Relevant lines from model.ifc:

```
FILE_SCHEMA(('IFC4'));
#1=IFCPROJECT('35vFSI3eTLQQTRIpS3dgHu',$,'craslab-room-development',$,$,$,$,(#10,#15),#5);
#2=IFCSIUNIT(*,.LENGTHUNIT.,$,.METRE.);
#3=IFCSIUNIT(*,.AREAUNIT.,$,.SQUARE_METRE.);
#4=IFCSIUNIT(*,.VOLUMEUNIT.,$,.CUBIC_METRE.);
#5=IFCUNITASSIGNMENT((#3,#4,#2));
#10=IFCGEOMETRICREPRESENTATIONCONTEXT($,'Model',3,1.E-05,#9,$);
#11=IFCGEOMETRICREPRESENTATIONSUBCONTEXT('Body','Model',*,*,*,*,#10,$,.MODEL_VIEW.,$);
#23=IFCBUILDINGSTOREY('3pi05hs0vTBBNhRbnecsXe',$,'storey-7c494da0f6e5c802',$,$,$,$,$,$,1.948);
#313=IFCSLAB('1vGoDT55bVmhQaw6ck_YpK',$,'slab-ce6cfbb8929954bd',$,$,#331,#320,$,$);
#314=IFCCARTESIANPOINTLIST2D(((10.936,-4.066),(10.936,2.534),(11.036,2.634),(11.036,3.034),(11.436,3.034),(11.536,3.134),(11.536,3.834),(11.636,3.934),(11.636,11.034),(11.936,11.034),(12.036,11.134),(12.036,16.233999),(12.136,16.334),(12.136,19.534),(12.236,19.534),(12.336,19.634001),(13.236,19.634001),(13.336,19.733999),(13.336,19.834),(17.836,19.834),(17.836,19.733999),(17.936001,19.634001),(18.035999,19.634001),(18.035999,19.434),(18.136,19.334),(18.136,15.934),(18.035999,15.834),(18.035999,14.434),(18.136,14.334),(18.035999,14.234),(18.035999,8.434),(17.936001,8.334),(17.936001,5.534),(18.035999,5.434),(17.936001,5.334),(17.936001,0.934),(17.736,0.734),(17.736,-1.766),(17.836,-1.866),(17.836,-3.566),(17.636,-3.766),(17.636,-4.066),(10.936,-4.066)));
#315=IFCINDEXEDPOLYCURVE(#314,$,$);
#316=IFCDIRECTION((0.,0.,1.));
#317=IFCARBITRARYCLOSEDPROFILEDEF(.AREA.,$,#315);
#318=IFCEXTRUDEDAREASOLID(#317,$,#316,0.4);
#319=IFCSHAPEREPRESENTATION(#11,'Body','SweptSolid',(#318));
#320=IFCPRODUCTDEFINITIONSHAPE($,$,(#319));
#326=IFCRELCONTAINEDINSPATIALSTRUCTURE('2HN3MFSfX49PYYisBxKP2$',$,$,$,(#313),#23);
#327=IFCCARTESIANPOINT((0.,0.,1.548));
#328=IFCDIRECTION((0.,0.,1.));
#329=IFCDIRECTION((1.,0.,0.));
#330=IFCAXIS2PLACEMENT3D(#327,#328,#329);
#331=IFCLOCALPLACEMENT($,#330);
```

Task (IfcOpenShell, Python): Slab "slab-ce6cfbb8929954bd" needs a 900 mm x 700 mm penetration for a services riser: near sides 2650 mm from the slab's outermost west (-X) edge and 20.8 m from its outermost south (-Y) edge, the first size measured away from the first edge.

```python
import numpy as np
import ifcopenshell
import ifcopenshell.api.feature
import ifcopenshell.api.geometry
import ifcopenshell.api.root
import ifcopenshell.geom
import ifcopenshell.util.placement
import ifcopenshell.util.representation
import ifcopenshell.util.shape
import ifcopenshell.util.unit

model = ifcopenshell.open("model.ifc")
unit_scale = ifcopenshell.util.unit.calculate_unit_scale(model)
settings = ifcopenshell.geom.settings()


def volume(element):
    """Net volume in cubic metres, openings subtracted."""
    shape = ifcopenshell.geom.create_shape(settings, element)
    return ifcopenshell.util.shape.get_volume(shape.geometry)


slab = model.by_id(313)
before = volume(slab)

# Extent in the slab's own axes, in metres. The edges named are its -X and -Y sides.
slab_shape = ifcopenshell.geom.create_shape(settings, slab)
vertices = ifcopenshell.util.shape.get_vertices(slab_shape.geometry)
x_min, y_min, bottom = vertices.min(axis=0)
top = vertices[:, 2].max()

opening = ifcopenshell.api.root.create_entity(model, ifc_class="IfcOpeningElement", name="Services riser opening", predefined_type="OPENING")
context = ifcopenshell.util.representation.get_context(model, "Model", "Body", "MODEL_VIEW")
width, depth = 0.9, 0.7
outline = [(0.0, 0.0), (width, 0.0), (width, depth), (0.0, depth), (0.0, 0.0)]
# Overshoot both faces by 50 mm so the cut is clean.
shape = ifcopenshell.api.geometry.add_slab_representation(
    model, context=context, depth=top - bottom + 0.1, polyline=outline
)
ifcopenshell.api.geometry.assign_representation(model, product=opening, representation=shape)

matrix = ifcopenshell.util.placement.get_local_placement(slab.ObjectPlacement)
matrix[:, 3] = matrix @ np.append(np.array([x_min + 2.65, y_min + 20.8, bottom - 0.05]) / unit_scale, 1.0)
ifcopenshell.api.geometry.edit_object_placement(model, product=opening, matrix=matrix, is_si=False)
ifcopenshell.api.feature.add_feature(model, feature=opening, element=slab)

after = volume(slab)

print(f"slab volume {before:.3f} -> {after:.3f} m3")

model.write("model-out.ifc")
```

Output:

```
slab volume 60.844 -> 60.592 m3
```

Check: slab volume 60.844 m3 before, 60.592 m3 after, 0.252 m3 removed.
